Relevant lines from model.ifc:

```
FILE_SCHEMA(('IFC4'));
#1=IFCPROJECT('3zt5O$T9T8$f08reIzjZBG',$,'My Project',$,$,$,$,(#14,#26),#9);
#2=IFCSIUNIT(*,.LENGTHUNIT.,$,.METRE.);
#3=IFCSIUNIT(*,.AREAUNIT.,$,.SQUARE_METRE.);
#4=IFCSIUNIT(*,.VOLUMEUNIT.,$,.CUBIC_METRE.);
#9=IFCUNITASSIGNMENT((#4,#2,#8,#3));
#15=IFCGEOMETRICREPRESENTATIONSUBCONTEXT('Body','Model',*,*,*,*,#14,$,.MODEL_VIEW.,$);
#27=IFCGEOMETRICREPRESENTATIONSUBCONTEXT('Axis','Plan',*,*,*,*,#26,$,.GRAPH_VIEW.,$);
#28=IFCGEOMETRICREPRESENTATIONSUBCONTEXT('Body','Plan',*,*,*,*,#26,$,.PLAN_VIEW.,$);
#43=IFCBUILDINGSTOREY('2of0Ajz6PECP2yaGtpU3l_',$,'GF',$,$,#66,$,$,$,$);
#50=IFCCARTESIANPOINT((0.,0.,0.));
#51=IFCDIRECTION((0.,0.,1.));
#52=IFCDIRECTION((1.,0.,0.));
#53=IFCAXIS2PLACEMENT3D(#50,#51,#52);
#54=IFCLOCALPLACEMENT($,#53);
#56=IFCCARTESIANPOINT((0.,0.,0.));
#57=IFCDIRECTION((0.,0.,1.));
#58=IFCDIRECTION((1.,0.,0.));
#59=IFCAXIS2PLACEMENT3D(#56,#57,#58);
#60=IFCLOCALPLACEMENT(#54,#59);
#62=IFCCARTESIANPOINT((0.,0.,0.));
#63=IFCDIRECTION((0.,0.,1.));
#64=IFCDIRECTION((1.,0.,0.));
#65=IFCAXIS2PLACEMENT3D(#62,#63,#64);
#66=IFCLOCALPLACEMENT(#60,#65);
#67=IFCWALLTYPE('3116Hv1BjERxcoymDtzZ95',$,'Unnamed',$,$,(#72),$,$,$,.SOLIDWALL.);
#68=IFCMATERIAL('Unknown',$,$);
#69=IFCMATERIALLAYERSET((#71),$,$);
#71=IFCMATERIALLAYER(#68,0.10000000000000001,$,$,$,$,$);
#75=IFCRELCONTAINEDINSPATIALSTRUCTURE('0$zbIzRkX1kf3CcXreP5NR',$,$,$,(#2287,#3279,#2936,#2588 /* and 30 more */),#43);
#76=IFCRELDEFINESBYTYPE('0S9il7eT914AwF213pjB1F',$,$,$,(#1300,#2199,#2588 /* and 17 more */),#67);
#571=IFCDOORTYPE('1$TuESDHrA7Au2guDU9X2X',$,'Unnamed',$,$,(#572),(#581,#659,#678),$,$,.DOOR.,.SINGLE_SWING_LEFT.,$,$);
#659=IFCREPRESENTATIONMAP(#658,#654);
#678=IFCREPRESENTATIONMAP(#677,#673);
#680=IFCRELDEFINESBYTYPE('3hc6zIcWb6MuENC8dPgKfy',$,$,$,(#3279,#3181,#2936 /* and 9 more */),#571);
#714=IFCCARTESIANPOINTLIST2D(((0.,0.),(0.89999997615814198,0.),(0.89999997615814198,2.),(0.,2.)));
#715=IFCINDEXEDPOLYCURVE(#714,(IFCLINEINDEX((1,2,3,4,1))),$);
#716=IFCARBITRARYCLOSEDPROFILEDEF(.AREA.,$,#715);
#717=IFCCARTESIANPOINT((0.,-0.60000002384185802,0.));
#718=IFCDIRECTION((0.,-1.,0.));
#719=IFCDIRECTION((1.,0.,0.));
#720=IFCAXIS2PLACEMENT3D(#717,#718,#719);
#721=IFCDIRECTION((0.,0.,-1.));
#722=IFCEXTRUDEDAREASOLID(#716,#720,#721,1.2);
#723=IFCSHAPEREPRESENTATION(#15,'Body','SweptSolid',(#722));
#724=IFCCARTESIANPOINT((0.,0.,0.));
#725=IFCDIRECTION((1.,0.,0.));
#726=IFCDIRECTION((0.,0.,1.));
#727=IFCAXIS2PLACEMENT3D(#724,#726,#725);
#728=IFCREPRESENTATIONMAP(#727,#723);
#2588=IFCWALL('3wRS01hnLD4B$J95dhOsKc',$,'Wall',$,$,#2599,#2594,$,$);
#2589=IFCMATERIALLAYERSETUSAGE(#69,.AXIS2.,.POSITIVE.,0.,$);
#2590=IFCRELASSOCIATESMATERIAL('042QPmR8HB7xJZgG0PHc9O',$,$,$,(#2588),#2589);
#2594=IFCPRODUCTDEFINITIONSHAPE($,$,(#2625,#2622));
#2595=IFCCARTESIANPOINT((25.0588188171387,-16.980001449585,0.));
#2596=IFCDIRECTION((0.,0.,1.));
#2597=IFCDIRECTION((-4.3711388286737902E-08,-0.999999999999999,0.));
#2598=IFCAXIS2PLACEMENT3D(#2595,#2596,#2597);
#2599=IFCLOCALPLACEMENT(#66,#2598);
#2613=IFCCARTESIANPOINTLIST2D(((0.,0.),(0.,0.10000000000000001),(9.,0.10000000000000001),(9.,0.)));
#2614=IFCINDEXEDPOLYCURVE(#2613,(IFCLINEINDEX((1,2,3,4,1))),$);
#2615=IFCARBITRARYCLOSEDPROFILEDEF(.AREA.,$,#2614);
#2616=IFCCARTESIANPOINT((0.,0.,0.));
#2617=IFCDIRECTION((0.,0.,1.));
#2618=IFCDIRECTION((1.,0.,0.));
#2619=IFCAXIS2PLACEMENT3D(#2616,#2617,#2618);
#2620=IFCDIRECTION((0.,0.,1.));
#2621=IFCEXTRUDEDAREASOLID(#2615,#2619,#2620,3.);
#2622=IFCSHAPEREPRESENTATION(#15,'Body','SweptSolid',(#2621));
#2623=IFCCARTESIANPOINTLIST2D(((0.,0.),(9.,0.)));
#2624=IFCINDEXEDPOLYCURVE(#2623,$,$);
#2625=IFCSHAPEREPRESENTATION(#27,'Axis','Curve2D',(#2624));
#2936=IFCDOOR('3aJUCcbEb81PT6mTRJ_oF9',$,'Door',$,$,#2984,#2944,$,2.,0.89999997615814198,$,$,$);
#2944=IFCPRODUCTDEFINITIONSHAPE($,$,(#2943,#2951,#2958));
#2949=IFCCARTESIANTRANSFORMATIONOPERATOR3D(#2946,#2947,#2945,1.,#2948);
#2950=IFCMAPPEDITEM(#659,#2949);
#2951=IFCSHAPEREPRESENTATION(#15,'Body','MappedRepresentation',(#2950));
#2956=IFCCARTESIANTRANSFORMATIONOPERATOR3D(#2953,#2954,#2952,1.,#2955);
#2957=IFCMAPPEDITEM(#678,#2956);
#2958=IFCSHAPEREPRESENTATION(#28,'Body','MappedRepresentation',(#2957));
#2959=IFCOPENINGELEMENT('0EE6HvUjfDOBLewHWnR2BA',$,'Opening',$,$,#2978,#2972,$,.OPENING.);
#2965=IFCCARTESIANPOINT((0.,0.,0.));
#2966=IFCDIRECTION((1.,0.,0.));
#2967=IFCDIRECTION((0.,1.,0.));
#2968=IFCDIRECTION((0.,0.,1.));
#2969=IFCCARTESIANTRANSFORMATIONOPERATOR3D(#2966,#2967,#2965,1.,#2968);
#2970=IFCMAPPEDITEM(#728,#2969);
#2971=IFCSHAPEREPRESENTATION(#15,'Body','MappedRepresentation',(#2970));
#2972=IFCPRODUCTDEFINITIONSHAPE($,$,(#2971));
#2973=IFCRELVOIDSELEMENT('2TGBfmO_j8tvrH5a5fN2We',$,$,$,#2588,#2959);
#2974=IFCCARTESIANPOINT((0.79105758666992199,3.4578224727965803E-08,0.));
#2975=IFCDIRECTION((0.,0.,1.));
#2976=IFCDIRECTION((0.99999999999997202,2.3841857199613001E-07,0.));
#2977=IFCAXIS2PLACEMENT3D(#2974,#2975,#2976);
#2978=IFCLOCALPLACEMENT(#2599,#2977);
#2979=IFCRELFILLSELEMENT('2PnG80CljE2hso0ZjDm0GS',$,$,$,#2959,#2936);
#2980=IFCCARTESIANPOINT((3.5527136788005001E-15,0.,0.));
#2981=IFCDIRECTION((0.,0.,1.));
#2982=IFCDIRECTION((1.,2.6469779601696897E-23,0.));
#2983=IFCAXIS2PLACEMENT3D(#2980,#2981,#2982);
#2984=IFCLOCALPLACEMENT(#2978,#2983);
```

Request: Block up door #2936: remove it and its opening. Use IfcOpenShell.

```python
import ifcopenshell
import ifcopenshell.api.feature
import ifcopenshell.api.root
import ifcopenshell.geom
import ifcopenshell.util.shape

model = ifcopenshell.open("model.ifc")
settings = ifcopenshell.geom.settings()


def volume(element):
    """Net volume in cubic metres, openings subtracted."""
    shape = ifcopenshell.geom.create_shape(settings, element)
    return ifcopenshell.util.shape.get_volume(shape.geometry)


door = model.by_id(2936)
opening = door.FillsVoids[0].RelatingOpeningElement
wall = opening.VoidsElements[0].RelatingBuildingElement
before = volume(wall)

ifcopenshell.api.root.remove_product(model, product=door)
ifcopenshell.api.feature.remove_feature(model, feature=opening)

after = volume(wall)

print(f"wall volume {before:.3f} -> {after:.3f} m3")

model.write("model_edited.ifc")
```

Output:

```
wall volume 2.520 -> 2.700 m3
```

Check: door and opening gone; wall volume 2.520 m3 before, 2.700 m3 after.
